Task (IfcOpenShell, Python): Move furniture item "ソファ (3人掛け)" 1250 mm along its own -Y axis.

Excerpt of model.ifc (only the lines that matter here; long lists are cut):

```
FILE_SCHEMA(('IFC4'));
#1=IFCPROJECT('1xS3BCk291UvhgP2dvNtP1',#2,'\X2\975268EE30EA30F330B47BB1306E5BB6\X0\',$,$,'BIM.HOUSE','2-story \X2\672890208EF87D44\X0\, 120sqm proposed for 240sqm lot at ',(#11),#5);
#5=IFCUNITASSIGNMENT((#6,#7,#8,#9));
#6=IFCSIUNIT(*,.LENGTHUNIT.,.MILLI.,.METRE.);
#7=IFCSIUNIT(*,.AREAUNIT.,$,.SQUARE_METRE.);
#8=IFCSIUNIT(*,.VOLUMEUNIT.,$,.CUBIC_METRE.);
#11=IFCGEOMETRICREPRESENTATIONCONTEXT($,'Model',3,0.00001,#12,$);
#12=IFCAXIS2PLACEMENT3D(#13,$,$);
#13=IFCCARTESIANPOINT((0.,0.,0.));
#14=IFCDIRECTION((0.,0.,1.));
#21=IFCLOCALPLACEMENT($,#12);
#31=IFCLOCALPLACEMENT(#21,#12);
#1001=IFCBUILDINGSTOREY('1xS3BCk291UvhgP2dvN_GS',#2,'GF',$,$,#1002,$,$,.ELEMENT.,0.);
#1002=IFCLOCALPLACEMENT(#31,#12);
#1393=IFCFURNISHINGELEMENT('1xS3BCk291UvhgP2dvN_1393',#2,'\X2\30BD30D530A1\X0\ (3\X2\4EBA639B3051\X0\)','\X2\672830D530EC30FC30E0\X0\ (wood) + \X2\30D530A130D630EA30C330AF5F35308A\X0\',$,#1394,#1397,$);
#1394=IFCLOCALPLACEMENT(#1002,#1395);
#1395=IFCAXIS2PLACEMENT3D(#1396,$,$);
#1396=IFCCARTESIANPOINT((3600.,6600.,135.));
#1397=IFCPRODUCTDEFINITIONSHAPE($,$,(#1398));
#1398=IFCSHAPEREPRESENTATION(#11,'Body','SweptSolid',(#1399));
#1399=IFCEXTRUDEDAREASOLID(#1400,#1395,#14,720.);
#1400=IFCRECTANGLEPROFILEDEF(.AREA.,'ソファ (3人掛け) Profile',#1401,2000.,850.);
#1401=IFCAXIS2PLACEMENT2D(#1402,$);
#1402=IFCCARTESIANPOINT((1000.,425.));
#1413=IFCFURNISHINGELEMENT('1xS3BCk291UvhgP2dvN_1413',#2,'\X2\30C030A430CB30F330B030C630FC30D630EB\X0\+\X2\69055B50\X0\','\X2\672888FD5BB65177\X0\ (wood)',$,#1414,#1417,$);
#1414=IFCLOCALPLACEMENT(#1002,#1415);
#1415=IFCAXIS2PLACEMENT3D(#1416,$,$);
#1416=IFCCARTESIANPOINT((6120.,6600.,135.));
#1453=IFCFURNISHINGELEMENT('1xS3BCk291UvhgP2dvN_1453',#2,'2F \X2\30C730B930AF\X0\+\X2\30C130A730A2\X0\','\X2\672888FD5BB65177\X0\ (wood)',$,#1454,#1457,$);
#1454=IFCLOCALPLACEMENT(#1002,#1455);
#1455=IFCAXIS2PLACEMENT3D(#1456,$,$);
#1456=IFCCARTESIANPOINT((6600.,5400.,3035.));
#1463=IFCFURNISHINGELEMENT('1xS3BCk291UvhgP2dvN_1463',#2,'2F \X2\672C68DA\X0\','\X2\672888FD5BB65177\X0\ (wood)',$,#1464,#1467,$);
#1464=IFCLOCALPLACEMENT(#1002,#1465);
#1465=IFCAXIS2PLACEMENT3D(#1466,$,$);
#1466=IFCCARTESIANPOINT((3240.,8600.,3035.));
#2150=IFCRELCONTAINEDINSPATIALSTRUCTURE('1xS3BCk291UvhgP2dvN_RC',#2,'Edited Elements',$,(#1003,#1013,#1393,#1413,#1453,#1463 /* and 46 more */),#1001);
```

```python
import ifcopenshell
import ifcopenshell.api.geometry
import ifcopenshell.util.placement
import ifcopenshell.util.unit

model = ifcopenshell.open("model.ifc")
unit_scale = ifcopenshell.util.unit.calculate_unit_scale(model)

item = model.by_guid("1xS3BCk291UvhgP2dvN_1393")
matrix = ifcopenshell.util.placement.get_local_placement(item.ObjectPlacement)
matrix[:3, 3] -= matrix[:3, 1] * 1.25 / unit_scale
ifcopenshell.api.geometry.edit_object_placement(model, product=item, matrix=matrix, is_si=False)

print(ifcopenshell.util.placement.get_local_placement(item.ObjectPlacement).round(3) + 0.0)

model.write("model-out.ifc")
```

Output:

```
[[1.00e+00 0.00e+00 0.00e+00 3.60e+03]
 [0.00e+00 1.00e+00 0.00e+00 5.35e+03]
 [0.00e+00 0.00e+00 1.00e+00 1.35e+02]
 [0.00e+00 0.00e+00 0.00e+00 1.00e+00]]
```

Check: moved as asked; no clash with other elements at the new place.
